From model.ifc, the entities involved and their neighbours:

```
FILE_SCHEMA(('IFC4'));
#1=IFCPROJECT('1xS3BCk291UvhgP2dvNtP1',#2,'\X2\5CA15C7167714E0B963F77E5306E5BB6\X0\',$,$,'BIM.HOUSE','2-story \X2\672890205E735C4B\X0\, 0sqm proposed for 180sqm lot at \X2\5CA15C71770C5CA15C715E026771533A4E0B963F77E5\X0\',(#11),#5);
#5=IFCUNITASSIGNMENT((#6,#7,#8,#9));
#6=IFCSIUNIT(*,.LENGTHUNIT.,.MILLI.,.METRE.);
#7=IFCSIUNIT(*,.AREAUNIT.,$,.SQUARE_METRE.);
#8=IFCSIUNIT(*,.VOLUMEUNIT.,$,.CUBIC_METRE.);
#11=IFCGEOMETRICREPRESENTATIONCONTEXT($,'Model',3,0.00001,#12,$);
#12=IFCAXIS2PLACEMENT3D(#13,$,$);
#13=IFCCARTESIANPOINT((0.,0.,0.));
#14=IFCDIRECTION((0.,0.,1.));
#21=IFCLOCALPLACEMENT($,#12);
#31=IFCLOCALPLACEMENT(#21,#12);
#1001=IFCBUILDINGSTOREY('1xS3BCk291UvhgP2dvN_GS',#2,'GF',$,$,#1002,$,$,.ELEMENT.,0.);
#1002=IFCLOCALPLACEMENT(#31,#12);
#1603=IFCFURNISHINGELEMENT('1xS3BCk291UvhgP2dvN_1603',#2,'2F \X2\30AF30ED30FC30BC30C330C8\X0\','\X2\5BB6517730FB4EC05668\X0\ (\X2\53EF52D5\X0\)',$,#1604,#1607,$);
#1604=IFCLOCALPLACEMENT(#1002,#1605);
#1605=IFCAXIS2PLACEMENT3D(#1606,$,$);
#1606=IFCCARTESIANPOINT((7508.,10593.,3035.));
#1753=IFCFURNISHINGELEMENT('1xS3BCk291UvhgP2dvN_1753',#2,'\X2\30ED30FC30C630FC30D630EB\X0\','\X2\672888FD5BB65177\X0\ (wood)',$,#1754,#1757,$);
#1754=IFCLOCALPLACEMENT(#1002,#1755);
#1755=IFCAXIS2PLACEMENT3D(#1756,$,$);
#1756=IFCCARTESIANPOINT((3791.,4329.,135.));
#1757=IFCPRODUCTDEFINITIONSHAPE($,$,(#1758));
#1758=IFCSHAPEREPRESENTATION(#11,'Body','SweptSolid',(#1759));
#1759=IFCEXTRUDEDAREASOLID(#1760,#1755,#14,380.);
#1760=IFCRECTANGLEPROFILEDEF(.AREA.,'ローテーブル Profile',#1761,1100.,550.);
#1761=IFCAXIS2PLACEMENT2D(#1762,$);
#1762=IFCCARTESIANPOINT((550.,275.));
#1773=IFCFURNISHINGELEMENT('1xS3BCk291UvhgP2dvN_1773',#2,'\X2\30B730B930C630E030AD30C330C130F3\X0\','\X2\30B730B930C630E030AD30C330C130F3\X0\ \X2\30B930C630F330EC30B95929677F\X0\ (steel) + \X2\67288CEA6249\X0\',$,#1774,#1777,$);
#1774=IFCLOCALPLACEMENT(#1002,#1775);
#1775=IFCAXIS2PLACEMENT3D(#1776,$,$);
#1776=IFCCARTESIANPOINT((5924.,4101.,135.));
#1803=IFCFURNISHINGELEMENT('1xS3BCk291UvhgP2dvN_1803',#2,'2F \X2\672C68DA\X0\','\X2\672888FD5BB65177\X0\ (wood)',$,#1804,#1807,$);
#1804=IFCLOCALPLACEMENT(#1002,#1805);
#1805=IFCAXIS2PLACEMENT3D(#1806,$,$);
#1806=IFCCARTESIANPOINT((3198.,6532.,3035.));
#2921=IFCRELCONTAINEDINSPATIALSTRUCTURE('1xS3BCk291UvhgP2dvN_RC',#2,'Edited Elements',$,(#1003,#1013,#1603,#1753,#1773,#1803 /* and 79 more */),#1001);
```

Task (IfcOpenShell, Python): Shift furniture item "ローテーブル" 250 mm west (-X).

```python
import ifcopenshell
import ifcopenshell.api.geometry
import ifcopenshell.util.placement

model = ifcopenshell.open("model.ifc")

item = model.by_id(1753)
matrix = ifcopenshell.util.placement.get_local_placement(item.ObjectPlacement)
matrix[0, 3] -= 250.0
ifcopenshell.api.geometry.edit_object_placement(model, product=item, matrix=matrix, is_si=False)

print(ifcopenshell.util.placement.get_local_placement(item.ObjectPlacement).round(3) + 0.0)

model.write("model_edited.ifc")
```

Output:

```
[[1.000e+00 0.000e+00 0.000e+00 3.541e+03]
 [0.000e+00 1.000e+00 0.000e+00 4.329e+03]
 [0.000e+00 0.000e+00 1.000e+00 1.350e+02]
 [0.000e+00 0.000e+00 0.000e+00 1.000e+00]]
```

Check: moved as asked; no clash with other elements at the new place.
